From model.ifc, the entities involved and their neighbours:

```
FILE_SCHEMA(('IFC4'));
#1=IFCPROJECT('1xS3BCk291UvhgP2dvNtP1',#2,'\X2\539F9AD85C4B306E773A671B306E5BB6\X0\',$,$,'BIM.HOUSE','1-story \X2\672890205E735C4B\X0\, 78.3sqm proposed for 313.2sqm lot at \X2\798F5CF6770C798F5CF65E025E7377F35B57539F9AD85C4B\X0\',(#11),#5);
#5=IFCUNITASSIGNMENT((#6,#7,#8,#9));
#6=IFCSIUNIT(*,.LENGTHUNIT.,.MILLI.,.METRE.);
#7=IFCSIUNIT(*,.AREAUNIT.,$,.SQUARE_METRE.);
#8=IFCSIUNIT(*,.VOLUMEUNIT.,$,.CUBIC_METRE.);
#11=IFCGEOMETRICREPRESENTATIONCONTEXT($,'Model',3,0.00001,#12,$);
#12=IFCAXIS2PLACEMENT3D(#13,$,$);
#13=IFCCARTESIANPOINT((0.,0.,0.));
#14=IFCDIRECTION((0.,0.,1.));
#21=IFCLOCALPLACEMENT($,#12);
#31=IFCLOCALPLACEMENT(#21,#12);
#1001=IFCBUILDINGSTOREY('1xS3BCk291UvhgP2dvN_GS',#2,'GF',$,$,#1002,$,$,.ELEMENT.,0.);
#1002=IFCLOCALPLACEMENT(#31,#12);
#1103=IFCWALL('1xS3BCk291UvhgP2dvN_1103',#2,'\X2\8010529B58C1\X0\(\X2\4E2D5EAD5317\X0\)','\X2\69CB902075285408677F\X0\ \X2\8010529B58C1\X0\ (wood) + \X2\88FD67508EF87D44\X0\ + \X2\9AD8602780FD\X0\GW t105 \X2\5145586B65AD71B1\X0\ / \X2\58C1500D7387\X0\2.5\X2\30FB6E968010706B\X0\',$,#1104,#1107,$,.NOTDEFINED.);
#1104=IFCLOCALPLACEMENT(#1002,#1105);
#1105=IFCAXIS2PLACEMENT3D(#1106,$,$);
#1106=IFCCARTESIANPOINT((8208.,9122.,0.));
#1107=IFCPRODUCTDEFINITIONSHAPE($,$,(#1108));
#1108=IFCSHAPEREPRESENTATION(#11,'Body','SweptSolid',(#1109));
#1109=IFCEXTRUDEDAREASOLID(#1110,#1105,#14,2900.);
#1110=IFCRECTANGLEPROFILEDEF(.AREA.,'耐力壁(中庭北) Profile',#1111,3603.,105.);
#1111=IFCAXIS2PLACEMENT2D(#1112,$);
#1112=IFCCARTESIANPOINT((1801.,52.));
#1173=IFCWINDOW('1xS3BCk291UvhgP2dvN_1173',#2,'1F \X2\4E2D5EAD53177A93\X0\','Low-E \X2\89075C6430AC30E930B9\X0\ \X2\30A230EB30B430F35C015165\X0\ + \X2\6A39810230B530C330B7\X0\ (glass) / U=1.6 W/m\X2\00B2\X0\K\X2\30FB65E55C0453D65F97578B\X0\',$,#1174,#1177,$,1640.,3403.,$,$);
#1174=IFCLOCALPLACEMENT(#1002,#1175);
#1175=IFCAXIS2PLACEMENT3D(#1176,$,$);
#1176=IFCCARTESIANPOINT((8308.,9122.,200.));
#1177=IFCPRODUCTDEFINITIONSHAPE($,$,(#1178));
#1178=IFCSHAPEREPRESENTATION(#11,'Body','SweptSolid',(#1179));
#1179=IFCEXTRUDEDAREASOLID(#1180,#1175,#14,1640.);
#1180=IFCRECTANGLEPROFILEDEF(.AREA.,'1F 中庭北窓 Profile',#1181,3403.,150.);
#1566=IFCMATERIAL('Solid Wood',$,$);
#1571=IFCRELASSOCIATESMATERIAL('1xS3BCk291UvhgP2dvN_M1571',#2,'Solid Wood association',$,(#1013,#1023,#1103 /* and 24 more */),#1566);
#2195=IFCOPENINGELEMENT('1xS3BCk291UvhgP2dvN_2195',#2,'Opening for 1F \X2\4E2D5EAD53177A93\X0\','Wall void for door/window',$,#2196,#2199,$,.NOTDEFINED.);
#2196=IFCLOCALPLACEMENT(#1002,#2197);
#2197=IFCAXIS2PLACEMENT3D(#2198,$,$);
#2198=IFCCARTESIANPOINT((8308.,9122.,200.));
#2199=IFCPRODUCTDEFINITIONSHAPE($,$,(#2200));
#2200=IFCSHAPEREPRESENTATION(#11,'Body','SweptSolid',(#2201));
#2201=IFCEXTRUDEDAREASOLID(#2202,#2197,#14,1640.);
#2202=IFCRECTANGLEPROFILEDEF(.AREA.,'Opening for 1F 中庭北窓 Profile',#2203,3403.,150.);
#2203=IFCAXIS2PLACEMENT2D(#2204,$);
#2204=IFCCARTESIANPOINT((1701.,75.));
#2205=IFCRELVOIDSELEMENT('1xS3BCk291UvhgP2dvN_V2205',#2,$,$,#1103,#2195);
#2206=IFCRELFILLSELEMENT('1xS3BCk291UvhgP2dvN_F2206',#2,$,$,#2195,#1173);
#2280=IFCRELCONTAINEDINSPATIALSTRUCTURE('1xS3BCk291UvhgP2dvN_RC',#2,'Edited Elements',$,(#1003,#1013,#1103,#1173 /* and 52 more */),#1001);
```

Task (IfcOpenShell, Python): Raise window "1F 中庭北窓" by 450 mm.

```python
import numpy as np
import ifcopenshell
import ifcopenshell.api.geometry
import ifcopenshell.util.placement
import ifcopenshell.util.unit

model = ifcopenshell.open("model.ifc")
unit_scale = ifcopenshell.util.unit.calculate_unit_scale(model)

window = model.by_guid("1xS3BCk291UvhgP2dvN_1173")
opening = window.FillsVoids[0].RelatingOpeningElement
dz = 0.45 / unit_scale

shift = np.array([0.0, 0.0, dz])
# The window is not placed relative to its opening, so move both.
for product in (opening, window):
    matrix = ifcopenshell.util.placement.get_local_placement(product.ObjectPlacement)
    matrix[:3, 3] += shift
    ifcopenshell.api.geometry.edit_object_placement(model, product=product, matrix=matrix, is_si=False)

print(f"moved by {dz * unit_scale:+.3f} m")

model.write("model-out.ifc")
```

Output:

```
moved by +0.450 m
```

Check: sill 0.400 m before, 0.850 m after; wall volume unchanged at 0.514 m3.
